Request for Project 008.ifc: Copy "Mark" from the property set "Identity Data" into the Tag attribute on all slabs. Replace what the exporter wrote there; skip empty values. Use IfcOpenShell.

First a look at what the model holds.

```python
import ifcopenshell
import ifcopenshell.util.element

model = ifcopenshell.open("Project 008.ifc")
print(model.schema)
slabs = model.by_type("IfcSlab")
print(len(slabs), "slabs")
for e in slabs[:8]:
    source = ifcopenshell.util.element.get_pset(e, "Identity Data", "Mark")
    target = e.Tag
    print(e.id(), repr(source), repr(target), sep=" | ")
```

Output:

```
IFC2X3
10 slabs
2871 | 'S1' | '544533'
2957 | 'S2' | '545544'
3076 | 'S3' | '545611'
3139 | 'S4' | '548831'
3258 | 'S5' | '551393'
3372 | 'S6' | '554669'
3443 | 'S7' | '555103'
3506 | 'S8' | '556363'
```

```python
import ifcopenshell
import ifcopenshell.util.element

model = ifcopenshell.open("Project 008.ifc")

count = 0
for e in model.by_type("IfcSlab"):
    value = ifcopenshell.util.element.get_pset(e, "Identity Data", "Mark")
    current = e.Tag
    if not value or not value.strip() or current == value:
        continue
    e.Tag = value
    count += 1

print(count, "slabs updated")

model.write("Project 008_rev.ifc")
```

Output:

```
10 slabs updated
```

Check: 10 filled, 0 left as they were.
